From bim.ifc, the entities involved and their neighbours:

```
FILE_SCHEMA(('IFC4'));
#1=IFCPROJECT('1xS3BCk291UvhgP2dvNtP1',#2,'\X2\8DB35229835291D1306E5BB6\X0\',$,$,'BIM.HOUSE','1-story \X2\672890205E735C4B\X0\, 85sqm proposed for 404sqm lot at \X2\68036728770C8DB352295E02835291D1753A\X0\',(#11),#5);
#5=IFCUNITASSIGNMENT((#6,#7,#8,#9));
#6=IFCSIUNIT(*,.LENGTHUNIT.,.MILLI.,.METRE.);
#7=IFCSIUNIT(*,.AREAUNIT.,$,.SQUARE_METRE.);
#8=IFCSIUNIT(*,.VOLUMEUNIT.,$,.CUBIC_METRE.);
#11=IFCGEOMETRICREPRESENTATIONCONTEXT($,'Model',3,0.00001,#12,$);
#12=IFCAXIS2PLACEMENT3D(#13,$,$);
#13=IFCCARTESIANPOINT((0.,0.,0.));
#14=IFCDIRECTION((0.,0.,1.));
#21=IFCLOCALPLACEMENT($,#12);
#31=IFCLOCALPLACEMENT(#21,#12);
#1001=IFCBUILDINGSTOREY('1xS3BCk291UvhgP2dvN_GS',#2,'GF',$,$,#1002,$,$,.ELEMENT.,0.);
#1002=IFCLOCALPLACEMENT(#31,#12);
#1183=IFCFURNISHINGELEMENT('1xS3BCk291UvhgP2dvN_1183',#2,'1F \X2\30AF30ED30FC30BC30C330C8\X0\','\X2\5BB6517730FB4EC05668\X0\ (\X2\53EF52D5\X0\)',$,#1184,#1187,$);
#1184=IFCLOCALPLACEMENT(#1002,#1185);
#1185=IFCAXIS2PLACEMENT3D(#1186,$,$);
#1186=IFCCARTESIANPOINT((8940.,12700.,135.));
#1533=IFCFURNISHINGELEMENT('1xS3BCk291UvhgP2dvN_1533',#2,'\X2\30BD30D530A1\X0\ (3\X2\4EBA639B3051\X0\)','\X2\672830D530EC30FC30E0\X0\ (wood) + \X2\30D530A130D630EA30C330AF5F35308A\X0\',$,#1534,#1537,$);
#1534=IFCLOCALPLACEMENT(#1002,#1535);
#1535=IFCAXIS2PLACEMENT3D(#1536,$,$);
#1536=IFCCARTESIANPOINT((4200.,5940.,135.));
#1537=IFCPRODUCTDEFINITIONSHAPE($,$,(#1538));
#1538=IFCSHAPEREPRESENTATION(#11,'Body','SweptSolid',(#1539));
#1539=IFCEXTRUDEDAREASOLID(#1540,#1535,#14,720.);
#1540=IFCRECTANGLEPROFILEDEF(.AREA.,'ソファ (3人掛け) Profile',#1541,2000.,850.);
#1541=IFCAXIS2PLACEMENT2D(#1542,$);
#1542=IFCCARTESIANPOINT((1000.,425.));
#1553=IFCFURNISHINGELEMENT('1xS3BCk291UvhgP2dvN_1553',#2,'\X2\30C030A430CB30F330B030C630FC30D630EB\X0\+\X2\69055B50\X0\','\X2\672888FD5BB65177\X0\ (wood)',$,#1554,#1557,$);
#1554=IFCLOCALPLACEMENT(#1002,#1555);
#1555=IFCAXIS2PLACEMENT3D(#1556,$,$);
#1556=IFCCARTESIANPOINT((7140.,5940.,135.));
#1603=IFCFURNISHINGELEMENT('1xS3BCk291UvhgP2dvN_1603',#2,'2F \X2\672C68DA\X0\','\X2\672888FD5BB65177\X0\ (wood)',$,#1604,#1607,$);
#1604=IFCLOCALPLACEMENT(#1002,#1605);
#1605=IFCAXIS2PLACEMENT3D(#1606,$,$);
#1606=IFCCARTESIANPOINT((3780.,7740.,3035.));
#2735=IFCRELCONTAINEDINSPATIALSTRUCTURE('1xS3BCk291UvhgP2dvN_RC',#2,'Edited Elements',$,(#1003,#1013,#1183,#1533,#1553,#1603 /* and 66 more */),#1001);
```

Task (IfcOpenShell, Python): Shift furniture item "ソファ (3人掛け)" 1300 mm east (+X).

```python
import ifcopenshell
import ifcopenshell.api.geometry
import ifcopenshell.util.placement
import ifcopenshell.util.unit

model = ifcopenshell.open("bim.ifc")
unit_scale = ifcopenshell.util.unit.calculate_unit_scale(model)

item = model.by_guid("1xS3BCk291UvhgP2dvN_1533")
matrix = ifcopenshell.util.placement.get_local_placement(item.ObjectPlacement)
matrix[0, 3] += 1.3 / unit_scale
ifcopenshell.api.geometry.edit_object_placement(model, product=item, matrix=matrix, is_si=False)

print(ifcopenshell.util.placement.get_local_placement(item.ObjectPlacement).round(3) + 0.0)

model.write("bim-out.ifc")
```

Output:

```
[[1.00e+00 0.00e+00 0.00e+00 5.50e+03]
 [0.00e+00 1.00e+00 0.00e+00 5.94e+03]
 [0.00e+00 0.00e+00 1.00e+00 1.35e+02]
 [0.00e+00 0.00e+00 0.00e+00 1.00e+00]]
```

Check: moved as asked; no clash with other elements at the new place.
